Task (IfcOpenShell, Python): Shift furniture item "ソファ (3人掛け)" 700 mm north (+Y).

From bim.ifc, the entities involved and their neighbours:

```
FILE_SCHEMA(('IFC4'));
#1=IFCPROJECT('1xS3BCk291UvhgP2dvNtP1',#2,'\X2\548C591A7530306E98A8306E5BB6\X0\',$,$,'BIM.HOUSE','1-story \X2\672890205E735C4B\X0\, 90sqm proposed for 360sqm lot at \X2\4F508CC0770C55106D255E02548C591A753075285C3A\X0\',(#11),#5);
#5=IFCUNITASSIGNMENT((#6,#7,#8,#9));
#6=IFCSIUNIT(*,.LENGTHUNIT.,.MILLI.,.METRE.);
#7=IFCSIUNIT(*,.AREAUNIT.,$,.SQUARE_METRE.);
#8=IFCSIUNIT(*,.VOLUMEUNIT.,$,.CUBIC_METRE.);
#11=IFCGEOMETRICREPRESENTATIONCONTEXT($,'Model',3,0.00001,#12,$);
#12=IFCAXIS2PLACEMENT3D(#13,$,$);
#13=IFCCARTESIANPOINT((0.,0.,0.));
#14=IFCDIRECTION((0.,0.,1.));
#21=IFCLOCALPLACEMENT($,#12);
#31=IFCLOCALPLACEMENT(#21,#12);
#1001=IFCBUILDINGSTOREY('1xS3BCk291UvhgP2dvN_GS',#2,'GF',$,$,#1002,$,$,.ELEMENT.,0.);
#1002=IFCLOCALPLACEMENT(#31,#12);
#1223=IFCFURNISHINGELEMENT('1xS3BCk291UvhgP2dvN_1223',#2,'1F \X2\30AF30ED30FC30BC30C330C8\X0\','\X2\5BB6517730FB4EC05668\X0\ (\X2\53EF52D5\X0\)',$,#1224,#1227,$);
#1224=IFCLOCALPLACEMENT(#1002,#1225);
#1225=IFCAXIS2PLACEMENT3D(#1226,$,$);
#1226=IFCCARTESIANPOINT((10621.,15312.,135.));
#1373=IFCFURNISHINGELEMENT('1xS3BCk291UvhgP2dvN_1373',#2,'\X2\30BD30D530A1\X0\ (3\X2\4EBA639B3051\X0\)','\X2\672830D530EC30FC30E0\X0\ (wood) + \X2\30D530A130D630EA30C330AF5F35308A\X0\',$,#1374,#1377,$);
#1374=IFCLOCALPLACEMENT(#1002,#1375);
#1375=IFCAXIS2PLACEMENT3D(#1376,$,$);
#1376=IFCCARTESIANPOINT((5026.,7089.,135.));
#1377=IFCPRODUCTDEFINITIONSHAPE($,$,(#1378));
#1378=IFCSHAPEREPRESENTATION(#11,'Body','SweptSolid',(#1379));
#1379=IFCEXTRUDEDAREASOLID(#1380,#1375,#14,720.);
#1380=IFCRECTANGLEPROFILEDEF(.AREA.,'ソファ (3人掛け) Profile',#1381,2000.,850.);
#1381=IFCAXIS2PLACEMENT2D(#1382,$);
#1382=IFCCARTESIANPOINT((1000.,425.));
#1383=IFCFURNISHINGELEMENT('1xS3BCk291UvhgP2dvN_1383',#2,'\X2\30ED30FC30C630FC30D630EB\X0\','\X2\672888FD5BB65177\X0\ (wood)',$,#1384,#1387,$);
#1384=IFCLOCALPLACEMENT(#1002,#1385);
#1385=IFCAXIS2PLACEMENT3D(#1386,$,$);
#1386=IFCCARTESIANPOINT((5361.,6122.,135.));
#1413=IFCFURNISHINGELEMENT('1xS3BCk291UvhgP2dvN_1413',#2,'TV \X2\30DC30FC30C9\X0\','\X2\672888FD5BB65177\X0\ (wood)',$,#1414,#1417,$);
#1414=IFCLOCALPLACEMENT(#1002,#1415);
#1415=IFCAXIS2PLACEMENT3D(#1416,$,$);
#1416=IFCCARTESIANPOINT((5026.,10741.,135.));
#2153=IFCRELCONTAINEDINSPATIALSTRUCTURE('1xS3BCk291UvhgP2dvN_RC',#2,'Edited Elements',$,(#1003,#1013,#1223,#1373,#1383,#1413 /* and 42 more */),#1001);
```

```python
import ifcopenshell
import ifcopenshell.api.geometry
import ifcopenshell.util.placement
import ifcopenshell.util.unit

model = ifcopenshell.open("bim.ifc")
unit_scale = ifcopenshell.util.unit.calculate_unit_scale(model)

item = model.by_id(1373)
matrix = ifcopenshell.util.placement.get_local_placement(item.ObjectPlacement)
matrix[1, 3] += 0.7 / unit_scale
ifcopenshell.api.geometry.edit_object_placement(model, product=item, matrix=matrix, is_si=False)

print(ifcopenshell.util.placement.get_local_placement(item.ObjectPlacement).round(3) + 0.0)

model.write("bim-out.ifc")
```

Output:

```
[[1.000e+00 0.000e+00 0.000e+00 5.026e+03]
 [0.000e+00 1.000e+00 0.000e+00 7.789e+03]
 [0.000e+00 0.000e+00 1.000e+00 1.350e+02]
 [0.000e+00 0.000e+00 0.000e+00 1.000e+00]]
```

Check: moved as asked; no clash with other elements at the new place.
